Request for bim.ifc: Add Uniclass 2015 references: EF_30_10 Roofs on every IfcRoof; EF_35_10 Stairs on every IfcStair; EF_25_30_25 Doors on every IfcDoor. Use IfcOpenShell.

First a look at what the model holds.

```python
import ifcopenshell

model = ifcopenshell.open("bim.ifc")
print(model.schema)
print("classifications:", [c.Name for c in model.by_type("IfcClassification")])
for ifc_class in ("IfcDoor", "IfcRoof", "IfcStair", "IfcWall", "IfcWindow"):
    print(ifc_class, len(model.by_type(ifc_class)))
```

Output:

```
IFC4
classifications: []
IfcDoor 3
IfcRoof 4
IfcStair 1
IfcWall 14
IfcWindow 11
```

```python
import ifcopenshell
import ifcopenshell.api.classification

model = ifcopenshell.open("bim.ifc")

system = ifcopenshell.api.classification.add_classification(model, classification="Uniclass 2015")

codes = {
    "IfcRoof": ("EF_30_10", "Roofs"),
    "IfcStair": ("EF_35_10", "Stairs"),
    "IfcDoor": ("EF_25_30_25", "Doors"),
}
for ifc_class, (code, name) in codes.items():
    products = model.by_type(ifc_class)
    ifcopenshell.api.classification.add_reference(
        model, products=products, classification=system, identification=code, name=name
    )
    print(code, len(products))

model.write("bim_rev.ifc")
```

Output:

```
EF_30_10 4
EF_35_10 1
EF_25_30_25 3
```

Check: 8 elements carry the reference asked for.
